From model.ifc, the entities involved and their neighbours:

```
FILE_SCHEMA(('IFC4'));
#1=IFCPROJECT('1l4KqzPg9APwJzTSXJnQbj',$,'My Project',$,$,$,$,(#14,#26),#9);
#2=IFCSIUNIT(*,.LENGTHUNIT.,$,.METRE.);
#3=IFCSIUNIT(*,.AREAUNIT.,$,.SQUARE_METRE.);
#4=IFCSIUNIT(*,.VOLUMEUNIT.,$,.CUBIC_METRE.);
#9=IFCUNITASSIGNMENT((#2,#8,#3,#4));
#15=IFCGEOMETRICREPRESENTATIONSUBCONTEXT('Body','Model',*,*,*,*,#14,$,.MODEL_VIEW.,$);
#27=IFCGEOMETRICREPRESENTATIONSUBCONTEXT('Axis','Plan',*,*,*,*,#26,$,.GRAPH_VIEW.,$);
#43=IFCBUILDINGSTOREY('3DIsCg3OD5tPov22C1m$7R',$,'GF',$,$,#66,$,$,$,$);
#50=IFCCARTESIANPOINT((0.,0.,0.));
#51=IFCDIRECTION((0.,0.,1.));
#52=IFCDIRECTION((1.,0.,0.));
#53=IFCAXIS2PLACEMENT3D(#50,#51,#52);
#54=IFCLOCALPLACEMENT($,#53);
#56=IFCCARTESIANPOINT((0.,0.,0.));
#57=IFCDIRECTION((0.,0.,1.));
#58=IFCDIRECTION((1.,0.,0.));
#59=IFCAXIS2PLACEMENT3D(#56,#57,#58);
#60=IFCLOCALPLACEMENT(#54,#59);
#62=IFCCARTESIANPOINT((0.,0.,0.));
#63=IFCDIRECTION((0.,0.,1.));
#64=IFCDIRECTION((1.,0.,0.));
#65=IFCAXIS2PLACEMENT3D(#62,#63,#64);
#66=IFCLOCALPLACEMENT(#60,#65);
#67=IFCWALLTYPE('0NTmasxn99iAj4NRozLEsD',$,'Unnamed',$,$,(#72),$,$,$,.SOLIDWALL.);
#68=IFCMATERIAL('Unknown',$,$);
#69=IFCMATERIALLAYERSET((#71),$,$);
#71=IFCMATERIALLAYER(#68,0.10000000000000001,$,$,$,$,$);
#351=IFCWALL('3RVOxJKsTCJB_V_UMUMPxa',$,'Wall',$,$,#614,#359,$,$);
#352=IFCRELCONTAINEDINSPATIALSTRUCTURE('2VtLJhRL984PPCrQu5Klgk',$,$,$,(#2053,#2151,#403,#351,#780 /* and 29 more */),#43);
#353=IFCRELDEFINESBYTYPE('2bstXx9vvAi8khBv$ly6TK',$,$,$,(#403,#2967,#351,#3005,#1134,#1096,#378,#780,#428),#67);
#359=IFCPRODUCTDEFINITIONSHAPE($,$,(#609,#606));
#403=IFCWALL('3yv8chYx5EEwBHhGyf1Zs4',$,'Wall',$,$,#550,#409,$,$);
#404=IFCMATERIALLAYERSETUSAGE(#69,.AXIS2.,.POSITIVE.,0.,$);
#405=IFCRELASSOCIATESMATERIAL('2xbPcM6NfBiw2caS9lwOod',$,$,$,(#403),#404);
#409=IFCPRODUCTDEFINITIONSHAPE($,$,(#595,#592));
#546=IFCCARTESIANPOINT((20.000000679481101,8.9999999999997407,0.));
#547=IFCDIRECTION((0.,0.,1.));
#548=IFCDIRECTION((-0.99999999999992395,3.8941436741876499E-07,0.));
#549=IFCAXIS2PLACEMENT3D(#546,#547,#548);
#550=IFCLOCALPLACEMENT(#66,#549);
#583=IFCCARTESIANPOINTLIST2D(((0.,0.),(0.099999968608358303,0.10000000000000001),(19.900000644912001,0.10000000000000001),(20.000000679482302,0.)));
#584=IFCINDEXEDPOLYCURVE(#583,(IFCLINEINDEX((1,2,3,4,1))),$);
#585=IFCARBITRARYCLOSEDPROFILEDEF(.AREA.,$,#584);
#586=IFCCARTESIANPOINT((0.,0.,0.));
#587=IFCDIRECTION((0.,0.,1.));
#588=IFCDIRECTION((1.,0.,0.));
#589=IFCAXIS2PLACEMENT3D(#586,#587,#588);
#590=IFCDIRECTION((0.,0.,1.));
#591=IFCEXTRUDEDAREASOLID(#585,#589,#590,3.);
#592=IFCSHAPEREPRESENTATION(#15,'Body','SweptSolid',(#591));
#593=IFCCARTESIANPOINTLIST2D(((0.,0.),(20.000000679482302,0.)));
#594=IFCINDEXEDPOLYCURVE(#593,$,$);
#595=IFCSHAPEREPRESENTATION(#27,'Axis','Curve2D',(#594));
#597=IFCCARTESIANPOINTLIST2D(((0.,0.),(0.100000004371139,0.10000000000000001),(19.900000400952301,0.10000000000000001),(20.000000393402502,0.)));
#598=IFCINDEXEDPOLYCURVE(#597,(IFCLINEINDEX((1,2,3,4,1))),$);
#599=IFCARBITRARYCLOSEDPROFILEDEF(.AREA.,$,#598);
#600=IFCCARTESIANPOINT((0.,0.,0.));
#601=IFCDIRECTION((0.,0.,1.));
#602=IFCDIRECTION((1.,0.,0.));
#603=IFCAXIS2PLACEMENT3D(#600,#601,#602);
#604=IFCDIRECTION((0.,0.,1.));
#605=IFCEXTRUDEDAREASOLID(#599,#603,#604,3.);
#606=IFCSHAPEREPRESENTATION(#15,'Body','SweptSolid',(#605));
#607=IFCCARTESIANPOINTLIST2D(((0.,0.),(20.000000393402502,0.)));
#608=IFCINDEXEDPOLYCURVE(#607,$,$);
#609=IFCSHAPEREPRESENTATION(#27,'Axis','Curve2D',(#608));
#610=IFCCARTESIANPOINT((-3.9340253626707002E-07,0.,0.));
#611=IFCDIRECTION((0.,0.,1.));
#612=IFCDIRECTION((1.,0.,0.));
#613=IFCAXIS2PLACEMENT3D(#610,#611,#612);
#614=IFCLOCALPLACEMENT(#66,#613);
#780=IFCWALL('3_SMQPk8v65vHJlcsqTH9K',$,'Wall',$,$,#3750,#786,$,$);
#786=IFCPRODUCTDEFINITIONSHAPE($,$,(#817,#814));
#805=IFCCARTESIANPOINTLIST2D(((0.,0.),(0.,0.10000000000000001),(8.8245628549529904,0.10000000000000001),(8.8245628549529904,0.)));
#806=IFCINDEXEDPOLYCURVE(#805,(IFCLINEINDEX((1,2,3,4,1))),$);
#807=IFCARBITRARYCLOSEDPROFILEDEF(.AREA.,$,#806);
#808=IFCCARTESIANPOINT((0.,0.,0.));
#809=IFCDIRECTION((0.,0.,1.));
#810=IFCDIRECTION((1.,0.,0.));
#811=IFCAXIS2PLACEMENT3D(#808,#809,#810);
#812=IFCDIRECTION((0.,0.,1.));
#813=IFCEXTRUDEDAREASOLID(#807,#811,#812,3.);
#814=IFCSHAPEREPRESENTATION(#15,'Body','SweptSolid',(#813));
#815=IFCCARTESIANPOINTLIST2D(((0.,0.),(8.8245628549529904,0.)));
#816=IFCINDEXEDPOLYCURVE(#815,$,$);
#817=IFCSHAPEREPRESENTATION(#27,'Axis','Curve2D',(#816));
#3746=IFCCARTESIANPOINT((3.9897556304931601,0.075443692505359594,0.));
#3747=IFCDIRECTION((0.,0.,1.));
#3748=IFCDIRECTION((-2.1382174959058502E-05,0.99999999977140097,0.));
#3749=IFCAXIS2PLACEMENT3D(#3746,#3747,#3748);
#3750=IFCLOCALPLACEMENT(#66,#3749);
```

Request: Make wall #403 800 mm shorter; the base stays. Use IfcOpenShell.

```python
import ifcopenshell
import ifcopenshell.geom
import ifcopenshell.util.representation
import ifcopenshell.util.shape

model = ifcopenshell.open("model.ifc")
settings = ifcopenshell.geom.settings()


def volume(element):
    """Net volume in cubic metres, openings subtracted."""
    shape = ifcopenshell.geom.create_shape(settings, element)
    return ifcopenshell.util.shape.get_volume(shape.geometry)


wall = model.by_guid("3yv8chYx5EEwBHhGyf1Zs4")
before = volume(wall)

body = ifcopenshell.util.representation.get_representation(wall, "Model", "Body")
solid = body.Items[0]
old_height = solid.Depth
solid.Depth -= 0.8
after = volume(wall)

print(f"height {old_height:g} -> {solid.Depth:g}, volume {before:.3f} -> {after:.3f} m3")

model.write("model_edited.ifc")
```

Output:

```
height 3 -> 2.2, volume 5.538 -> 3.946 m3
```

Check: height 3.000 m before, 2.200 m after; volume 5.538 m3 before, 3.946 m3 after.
